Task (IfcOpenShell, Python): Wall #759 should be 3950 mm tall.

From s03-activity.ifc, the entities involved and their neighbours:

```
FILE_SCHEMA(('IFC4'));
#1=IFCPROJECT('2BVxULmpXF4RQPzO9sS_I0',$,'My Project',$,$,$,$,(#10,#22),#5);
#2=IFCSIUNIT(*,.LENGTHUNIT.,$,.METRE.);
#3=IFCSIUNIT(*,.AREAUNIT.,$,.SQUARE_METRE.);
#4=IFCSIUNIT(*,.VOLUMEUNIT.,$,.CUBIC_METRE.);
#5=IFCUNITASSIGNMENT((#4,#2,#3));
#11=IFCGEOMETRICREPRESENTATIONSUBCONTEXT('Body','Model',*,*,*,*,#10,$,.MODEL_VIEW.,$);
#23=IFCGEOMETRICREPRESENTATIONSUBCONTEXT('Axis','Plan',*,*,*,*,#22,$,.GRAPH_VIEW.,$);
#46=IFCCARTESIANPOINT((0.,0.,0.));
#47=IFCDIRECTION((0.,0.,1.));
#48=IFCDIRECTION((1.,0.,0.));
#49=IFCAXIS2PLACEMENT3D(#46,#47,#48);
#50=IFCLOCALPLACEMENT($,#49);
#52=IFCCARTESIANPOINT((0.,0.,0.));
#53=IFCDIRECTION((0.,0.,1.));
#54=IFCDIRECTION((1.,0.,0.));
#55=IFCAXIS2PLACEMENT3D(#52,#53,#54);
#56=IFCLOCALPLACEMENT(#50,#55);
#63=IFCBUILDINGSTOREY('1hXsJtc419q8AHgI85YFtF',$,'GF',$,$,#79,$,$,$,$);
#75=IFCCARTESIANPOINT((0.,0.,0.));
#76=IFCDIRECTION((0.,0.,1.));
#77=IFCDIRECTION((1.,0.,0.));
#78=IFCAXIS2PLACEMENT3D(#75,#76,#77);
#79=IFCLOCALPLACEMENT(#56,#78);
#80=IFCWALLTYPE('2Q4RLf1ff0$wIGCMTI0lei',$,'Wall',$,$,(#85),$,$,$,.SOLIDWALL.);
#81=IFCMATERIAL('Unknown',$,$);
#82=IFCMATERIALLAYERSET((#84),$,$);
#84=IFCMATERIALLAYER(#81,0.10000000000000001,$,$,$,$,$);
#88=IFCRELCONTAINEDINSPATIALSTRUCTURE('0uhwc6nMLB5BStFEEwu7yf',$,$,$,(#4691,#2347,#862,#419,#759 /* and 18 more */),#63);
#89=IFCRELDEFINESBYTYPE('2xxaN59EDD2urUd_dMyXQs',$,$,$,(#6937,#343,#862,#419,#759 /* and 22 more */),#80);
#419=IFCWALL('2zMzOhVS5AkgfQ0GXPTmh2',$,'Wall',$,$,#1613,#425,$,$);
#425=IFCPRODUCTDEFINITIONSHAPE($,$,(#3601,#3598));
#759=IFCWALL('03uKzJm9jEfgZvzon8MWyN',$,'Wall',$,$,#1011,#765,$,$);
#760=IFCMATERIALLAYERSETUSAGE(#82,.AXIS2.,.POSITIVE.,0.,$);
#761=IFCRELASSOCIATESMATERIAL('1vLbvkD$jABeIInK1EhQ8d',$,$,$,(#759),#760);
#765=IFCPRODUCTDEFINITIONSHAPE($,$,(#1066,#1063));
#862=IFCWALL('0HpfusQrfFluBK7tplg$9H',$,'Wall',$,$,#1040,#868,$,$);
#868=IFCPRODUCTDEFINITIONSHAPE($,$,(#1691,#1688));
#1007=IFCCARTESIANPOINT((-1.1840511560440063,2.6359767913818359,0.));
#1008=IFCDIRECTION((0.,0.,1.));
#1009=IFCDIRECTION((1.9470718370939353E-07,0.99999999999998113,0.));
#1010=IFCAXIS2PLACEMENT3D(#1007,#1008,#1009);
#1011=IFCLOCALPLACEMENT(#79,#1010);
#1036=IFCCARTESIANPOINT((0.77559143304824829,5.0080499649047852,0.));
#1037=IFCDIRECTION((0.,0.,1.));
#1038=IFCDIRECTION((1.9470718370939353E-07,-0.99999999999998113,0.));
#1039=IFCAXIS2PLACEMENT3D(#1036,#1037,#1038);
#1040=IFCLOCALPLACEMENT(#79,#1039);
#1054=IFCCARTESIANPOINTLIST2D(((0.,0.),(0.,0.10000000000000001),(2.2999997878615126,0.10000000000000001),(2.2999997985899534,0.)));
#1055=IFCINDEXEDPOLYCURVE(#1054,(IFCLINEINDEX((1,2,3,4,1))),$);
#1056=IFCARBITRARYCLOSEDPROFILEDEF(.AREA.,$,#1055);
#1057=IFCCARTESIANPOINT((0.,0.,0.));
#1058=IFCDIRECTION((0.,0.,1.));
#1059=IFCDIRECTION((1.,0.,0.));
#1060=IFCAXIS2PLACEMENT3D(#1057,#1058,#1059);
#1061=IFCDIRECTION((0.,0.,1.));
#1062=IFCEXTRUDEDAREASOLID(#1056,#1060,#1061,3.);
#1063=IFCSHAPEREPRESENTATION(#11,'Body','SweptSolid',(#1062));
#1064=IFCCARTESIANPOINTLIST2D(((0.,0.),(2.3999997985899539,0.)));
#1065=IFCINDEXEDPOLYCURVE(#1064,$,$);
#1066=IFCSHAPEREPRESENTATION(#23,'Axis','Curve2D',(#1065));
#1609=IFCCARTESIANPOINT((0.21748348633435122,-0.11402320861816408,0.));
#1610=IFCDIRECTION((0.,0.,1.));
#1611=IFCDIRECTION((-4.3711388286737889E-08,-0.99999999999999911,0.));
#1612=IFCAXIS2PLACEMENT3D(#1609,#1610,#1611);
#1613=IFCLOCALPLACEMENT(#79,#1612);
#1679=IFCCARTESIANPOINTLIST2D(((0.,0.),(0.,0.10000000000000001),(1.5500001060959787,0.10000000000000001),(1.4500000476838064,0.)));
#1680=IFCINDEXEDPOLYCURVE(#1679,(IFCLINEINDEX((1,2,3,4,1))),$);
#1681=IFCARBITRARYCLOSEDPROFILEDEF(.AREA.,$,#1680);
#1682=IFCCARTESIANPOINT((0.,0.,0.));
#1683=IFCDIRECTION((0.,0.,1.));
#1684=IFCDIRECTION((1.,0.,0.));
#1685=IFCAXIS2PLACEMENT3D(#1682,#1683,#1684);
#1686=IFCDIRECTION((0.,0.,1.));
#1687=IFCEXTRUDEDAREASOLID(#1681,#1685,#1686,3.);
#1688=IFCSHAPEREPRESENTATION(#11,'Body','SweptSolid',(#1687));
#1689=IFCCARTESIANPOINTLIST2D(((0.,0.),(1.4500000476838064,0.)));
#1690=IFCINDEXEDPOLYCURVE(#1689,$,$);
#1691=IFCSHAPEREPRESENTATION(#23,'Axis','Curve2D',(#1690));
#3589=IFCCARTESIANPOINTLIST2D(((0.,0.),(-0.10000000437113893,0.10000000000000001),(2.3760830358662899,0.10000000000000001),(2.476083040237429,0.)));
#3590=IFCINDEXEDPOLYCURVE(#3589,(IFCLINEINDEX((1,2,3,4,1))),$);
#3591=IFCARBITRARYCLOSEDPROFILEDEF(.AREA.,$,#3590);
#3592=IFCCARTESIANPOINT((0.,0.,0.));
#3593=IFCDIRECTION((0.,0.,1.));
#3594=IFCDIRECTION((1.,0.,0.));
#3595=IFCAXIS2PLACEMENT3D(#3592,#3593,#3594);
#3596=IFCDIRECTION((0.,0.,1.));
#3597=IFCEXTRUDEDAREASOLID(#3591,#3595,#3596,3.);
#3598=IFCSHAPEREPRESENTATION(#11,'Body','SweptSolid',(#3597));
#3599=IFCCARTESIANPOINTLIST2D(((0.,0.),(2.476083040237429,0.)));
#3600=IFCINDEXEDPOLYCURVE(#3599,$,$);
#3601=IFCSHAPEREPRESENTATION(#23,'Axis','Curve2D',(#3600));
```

```python
import ifcopenshell
import ifcopenshell.geom
import ifcopenshell.util.representation
import ifcopenshell.util.shape
import ifcopenshell.util.unit

model = ifcopenshell.open("s03-activity.ifc")
unit_scale = ifcopenshell.util.unit.calculate_unit_scale(model)
settings = ifcopenshell.geom.settings()


def volume(element):
    """Net volume in cubic metres, openings subtracted."""
    shape = ifcopenshell.geom.create_shape(settings, element)
    return ifcopenshell.util.shape.get_volume(shape.geometry)


wall = model.by_id(759)
before = volume(wall)

body = ifcopenshell.util.representation.get_representation(wall, "Model", "Body")
solid = body.Items[0]
old_height = solid.Depth
solid.Depth = 3.95 / unit_scale
after = volume(wall)

print(f"height {old_height:g} -> {solid.Depth:g}, volume {before:.3f} -> {after:.3f} m3")

model.write("s03-activity-out.ifc")
```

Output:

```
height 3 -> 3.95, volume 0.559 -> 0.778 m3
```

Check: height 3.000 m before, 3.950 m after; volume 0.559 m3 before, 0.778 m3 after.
